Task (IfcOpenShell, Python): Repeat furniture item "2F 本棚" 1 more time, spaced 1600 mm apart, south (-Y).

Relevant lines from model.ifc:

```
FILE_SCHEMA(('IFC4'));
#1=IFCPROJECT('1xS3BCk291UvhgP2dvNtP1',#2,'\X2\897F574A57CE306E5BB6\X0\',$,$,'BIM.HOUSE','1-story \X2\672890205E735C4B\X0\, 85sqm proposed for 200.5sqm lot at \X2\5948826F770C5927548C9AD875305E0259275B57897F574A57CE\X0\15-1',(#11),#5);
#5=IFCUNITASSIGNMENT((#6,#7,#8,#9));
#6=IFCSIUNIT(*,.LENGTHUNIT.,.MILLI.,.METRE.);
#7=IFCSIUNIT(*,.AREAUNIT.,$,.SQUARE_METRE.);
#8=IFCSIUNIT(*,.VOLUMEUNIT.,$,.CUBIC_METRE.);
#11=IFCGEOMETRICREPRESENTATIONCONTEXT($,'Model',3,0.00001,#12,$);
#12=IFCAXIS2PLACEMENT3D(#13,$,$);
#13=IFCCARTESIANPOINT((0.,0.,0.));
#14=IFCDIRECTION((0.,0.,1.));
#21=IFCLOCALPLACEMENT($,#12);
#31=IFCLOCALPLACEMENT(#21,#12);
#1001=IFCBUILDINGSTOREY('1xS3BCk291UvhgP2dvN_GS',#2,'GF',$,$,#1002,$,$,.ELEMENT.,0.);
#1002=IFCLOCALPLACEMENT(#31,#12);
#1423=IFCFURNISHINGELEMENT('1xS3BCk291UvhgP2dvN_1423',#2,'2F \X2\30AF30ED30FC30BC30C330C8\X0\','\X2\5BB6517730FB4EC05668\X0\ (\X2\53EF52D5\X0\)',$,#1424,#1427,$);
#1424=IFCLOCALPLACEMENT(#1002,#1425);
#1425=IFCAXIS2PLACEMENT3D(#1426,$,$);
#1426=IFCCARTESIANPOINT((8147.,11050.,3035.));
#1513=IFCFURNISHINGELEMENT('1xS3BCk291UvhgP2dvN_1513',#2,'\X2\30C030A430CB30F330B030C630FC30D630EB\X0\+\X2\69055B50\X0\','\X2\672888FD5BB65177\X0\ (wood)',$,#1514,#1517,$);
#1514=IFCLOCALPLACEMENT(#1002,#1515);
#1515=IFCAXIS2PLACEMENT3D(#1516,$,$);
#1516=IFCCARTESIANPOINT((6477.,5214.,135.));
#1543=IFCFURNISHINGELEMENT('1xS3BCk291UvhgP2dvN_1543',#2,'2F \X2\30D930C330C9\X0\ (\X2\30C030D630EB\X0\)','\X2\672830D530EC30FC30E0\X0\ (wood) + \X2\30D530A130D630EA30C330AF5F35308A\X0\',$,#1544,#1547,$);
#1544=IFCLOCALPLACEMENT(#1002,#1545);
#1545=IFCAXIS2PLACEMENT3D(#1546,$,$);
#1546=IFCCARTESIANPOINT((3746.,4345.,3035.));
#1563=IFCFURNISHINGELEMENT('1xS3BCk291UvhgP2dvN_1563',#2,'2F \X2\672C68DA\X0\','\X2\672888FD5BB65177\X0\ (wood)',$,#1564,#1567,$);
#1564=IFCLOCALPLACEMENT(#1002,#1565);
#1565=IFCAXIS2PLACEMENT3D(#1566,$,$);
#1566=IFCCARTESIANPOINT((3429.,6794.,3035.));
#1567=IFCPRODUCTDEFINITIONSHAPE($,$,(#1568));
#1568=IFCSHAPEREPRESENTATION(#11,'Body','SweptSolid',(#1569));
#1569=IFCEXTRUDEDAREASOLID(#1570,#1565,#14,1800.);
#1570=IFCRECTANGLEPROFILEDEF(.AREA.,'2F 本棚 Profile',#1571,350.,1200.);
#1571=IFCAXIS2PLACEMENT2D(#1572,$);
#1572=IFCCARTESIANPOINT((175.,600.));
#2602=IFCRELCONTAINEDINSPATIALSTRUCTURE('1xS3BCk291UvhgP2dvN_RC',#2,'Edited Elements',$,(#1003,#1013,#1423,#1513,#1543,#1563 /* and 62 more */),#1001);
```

```python
import numpy as np
import ifcopenshell
import ifcopenshell.api.geometry
import ifcopenshell.api.root
import ifcopenshell.util.element
import ifcopenshell.util.placement
import ifcopenshell.util.unit

model = ifcopenshell.open("model.ifc")
unit_scale = ifcopenshell.util.unit.calculate_unit_scale(model)


def reuse_history(source, copy):
    """copy_class also copies each property set's owner history, people and application; keep the originals."""
    for rel in copy.IsDefinedBy:
        if rel.is_a("IfcRelDefinesByProperties") and (history := rel.RelatingPropertyDefinition.OwnerHistory):
            rel.RelatingPropertyDefinition.OwnerHistory = source.OwnerHistory
            ifcopenshell.util.element.remove_deep2(model, history)


source = model.by_id(1563)
base = ifcopenshell.util.placement.get_local_placement(source.ObjectPlacement)
step = np.array([0.0, -1.0, 0.0]) * 1.6 / unit_scale

for i in range(1, 2):
    copy = ifcopenshell.api.root.copy_class(model, product=source)
    copy.Representation = ifcopenshell.util.element.copy_deep(
        model, source.Representation, exclude=["IfcGeometricRepresentationContext", "IfcRepresentationMap"]
    )
    reuse_history(source, copy)
    matrix = base.copy()
    matrix[:3, 3] += i * step
    print("added at", matrix[:3, 3].round(3) + 0.0)
    ifcopenshell.api.geometry.edit_object_placement(model, product=copy, matrix=matrix, is_si=False)

model.write("model-out.ifc")
```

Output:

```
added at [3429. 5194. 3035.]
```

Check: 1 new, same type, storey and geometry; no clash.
